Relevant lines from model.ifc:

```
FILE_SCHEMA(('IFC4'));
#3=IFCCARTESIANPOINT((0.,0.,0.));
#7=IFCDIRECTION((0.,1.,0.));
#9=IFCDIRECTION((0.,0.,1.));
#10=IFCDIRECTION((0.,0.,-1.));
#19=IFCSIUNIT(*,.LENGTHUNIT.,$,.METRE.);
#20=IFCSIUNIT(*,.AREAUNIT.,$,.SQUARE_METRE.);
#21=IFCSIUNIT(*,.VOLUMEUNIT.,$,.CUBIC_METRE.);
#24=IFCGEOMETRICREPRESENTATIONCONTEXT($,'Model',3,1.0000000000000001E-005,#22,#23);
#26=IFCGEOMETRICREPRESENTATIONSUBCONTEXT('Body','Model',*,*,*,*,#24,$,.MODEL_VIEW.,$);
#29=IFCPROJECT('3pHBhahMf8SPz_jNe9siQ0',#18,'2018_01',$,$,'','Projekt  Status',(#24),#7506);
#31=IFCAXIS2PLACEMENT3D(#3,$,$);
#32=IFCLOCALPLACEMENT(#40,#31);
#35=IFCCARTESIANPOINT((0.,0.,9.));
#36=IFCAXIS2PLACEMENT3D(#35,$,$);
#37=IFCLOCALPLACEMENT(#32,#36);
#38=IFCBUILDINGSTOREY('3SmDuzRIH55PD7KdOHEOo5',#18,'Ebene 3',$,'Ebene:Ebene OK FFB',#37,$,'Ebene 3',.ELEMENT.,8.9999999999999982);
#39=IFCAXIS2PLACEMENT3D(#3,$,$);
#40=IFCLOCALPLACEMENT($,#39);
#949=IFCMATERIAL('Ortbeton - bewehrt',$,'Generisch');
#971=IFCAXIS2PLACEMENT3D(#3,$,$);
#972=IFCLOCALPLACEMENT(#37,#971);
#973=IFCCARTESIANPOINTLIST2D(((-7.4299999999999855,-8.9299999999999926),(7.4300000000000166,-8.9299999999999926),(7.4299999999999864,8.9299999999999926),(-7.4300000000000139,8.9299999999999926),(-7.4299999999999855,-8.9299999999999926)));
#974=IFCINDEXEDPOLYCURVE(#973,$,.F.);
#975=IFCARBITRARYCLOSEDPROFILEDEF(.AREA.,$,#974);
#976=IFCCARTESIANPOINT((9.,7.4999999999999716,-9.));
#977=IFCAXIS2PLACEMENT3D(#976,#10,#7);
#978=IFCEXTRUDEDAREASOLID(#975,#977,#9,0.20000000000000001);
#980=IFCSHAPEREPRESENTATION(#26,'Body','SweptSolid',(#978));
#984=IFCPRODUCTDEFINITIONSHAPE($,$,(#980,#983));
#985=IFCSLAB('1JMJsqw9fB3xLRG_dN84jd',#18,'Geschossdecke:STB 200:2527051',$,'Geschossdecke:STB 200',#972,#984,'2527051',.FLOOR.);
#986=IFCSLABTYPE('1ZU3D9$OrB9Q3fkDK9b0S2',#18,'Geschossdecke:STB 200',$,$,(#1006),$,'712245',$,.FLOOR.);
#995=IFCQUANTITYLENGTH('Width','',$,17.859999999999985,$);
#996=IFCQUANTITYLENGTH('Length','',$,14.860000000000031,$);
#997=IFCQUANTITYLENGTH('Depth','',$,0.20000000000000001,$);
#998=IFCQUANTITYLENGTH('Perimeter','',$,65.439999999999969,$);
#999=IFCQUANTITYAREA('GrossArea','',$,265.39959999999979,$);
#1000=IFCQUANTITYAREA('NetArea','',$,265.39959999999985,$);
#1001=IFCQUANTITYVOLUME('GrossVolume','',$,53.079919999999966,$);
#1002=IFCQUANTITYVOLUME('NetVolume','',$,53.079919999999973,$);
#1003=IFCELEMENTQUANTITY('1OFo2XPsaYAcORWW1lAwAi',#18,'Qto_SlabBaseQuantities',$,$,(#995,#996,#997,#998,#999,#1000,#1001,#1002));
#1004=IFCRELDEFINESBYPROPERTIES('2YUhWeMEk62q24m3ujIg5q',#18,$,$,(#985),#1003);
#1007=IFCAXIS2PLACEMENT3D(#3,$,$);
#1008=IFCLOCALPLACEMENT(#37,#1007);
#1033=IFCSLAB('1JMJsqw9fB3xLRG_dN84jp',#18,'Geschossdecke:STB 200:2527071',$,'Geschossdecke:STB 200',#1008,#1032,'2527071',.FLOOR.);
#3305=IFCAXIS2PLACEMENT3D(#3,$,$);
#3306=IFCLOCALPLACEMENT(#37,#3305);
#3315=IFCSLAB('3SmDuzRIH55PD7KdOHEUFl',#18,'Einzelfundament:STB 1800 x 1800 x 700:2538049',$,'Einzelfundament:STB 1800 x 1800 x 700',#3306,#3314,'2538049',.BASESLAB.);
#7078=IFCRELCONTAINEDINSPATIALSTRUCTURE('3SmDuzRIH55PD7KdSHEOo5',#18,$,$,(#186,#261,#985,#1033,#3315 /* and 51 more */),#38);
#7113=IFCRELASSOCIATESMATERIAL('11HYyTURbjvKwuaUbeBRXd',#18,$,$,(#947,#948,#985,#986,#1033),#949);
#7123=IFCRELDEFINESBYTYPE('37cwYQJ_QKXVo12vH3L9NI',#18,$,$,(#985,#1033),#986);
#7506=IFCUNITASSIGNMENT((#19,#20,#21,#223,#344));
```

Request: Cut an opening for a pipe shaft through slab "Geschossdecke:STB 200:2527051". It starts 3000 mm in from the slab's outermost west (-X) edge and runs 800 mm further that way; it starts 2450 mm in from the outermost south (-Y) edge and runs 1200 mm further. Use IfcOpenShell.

```python
import numpy as np
import ifcopenshell
import ifcopenshell.api.feature
import ifcopenshell.api.geometry
import ifcopenshell.api.pset
import ifcopenshell.api.root
import ifcopenshell.geom
import ifcopenshell.util.element
import ifcopenshell.util.placement
import ifcopenshell.util.representation
import ifcopenshell.util.shape
import ifcopenshell.util.unit

model = ifcopenshell.open("model.ifc")
unit_scale = ifcopenshell.util.unit.calculate_unit_scale(model)
area_scale = ifcopenshell.util.unit.calculate_unit_scale(model, "AREAUNIT")
volume_scale = ifcopenshell.util.unit.calculate_unit_scale(model, "VOLUMEUNIT")
settings = ifcopenshell.geom.settings()


def volume(element):
    """Net volume in cubic metres, openings subtracted."""
    shape = ifcopenshell.geom.create_shape(settings, element)
    return ifcopenshell.util.shape.get_volume(shape.geometry)


slab = model.by_guid("1JMJsqw9fB3xLRG_dN84jd")
before = volume(slab)

# Extent in the slab's own axes, in metres. The edges named are its -X and -Y sides.
slab_shape = ifcopenshell.geom.create_shape(settings, slab)
vertices = ifcopenshell.util.shape.get_vertices(slab_shape.geometry)
x_min, y_min, bottom = vertices.min(axis=0)
top = vertices[:, 2].max()

opening = ifcopenshell.api.root.create_entity(model, ifc_class="IfcOpeningElement", name="Pipe shaft opening", predefined_type="OPENING")
context = ifcopenshell.util.representation.get_context(model, "Model", "Body", "MODEL_VIEW")
width, depth = 0.8, 1.2
outline = [(0.0, 0.0), (width, 0.0), (width, depth), (0.0, depth), (0.0, 0.0)]
# Overshoot both faces by 50 mm so the cut is clean.
shape = ifcopenshell.api.geometry.add_slab_representation(
    model, context=context, depth=top - bottom + 0.1, polyline=outline
)
ifcopenshell.api.geometry.assign_representation(model, product=opening, representation=shape)

matrix = ifcopenshell.util.placement.get_local_placement(slab.ObjectPlacement)
matrix[:, 3] = matrix @ np.append(np.array([x_min + 3, y_min + 2.45, bottom - 0.05]) / unit_scale, 1.0)
ifcopenshell.api.geometry.edit_object_placement(model, product=opening, matrix=matrix, is_si=False)
ifcopenshell.api.feature.add_feature(model, feature=opening, element=slab)

after = volume(slab)

# Update the slab's stored quantities.
qto = model.by_id(ifcopenshell.util.element.get_pset(slab, "Qto_SlabBaseQuantities", should_inherit=False)["id"])
ifcopenshell.api.pset.edit_qto(model, qto=qto, properties={
    "NetArea": after / (top - bottom) / area_scale,
    "NetVolume": after / volume_scale,
})

print(f"slab volume {before:.3f} -> {after:.3f} m3")

model.write("model-out.ifc")
```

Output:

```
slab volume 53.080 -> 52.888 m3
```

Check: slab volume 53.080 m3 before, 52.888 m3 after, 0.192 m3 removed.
